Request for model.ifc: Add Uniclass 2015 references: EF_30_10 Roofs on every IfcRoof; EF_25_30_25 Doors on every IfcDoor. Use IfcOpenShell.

First a look at what the model holds.

```python
import ifcopenshell

model = ifcopenshell.open("model.ifc")
print(model.schema)
print("classifications:", [c.Name for c in model.by_type("IfcClassification")])
for ifc_class in ("IfcDoor", "IfcRoof", "IfcStair", "IfcWall", "IfcWindow"):
    print(ifc_class, len(model.by_type(ifc_class)))
```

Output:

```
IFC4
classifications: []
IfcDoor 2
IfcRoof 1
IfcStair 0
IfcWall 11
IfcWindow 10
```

```python
import ifcopenshell
import ifcopenshell.api.classification

model = ifcopenshell.open("model.ifc")

system = ifcopenshell.api.classification.add_classification(model, classification="Uniclass 2015")

codes = {
    "IfcRoof": ("EF_30_10", "Roofs"),
    "IfcDoor": ("EF_25_30_25", "Doors"),
}
for ifc_class, (code, name) in codes.items():
    products = model.by_type(ifc_class)
    ifcopenshell.api.classification.add_reference(
        model, products=products, classification=system, identification=code, name=name
    )
    print(code, len(products))

model.write("model_updated.ifc")
```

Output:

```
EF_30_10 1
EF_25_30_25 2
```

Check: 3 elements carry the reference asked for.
